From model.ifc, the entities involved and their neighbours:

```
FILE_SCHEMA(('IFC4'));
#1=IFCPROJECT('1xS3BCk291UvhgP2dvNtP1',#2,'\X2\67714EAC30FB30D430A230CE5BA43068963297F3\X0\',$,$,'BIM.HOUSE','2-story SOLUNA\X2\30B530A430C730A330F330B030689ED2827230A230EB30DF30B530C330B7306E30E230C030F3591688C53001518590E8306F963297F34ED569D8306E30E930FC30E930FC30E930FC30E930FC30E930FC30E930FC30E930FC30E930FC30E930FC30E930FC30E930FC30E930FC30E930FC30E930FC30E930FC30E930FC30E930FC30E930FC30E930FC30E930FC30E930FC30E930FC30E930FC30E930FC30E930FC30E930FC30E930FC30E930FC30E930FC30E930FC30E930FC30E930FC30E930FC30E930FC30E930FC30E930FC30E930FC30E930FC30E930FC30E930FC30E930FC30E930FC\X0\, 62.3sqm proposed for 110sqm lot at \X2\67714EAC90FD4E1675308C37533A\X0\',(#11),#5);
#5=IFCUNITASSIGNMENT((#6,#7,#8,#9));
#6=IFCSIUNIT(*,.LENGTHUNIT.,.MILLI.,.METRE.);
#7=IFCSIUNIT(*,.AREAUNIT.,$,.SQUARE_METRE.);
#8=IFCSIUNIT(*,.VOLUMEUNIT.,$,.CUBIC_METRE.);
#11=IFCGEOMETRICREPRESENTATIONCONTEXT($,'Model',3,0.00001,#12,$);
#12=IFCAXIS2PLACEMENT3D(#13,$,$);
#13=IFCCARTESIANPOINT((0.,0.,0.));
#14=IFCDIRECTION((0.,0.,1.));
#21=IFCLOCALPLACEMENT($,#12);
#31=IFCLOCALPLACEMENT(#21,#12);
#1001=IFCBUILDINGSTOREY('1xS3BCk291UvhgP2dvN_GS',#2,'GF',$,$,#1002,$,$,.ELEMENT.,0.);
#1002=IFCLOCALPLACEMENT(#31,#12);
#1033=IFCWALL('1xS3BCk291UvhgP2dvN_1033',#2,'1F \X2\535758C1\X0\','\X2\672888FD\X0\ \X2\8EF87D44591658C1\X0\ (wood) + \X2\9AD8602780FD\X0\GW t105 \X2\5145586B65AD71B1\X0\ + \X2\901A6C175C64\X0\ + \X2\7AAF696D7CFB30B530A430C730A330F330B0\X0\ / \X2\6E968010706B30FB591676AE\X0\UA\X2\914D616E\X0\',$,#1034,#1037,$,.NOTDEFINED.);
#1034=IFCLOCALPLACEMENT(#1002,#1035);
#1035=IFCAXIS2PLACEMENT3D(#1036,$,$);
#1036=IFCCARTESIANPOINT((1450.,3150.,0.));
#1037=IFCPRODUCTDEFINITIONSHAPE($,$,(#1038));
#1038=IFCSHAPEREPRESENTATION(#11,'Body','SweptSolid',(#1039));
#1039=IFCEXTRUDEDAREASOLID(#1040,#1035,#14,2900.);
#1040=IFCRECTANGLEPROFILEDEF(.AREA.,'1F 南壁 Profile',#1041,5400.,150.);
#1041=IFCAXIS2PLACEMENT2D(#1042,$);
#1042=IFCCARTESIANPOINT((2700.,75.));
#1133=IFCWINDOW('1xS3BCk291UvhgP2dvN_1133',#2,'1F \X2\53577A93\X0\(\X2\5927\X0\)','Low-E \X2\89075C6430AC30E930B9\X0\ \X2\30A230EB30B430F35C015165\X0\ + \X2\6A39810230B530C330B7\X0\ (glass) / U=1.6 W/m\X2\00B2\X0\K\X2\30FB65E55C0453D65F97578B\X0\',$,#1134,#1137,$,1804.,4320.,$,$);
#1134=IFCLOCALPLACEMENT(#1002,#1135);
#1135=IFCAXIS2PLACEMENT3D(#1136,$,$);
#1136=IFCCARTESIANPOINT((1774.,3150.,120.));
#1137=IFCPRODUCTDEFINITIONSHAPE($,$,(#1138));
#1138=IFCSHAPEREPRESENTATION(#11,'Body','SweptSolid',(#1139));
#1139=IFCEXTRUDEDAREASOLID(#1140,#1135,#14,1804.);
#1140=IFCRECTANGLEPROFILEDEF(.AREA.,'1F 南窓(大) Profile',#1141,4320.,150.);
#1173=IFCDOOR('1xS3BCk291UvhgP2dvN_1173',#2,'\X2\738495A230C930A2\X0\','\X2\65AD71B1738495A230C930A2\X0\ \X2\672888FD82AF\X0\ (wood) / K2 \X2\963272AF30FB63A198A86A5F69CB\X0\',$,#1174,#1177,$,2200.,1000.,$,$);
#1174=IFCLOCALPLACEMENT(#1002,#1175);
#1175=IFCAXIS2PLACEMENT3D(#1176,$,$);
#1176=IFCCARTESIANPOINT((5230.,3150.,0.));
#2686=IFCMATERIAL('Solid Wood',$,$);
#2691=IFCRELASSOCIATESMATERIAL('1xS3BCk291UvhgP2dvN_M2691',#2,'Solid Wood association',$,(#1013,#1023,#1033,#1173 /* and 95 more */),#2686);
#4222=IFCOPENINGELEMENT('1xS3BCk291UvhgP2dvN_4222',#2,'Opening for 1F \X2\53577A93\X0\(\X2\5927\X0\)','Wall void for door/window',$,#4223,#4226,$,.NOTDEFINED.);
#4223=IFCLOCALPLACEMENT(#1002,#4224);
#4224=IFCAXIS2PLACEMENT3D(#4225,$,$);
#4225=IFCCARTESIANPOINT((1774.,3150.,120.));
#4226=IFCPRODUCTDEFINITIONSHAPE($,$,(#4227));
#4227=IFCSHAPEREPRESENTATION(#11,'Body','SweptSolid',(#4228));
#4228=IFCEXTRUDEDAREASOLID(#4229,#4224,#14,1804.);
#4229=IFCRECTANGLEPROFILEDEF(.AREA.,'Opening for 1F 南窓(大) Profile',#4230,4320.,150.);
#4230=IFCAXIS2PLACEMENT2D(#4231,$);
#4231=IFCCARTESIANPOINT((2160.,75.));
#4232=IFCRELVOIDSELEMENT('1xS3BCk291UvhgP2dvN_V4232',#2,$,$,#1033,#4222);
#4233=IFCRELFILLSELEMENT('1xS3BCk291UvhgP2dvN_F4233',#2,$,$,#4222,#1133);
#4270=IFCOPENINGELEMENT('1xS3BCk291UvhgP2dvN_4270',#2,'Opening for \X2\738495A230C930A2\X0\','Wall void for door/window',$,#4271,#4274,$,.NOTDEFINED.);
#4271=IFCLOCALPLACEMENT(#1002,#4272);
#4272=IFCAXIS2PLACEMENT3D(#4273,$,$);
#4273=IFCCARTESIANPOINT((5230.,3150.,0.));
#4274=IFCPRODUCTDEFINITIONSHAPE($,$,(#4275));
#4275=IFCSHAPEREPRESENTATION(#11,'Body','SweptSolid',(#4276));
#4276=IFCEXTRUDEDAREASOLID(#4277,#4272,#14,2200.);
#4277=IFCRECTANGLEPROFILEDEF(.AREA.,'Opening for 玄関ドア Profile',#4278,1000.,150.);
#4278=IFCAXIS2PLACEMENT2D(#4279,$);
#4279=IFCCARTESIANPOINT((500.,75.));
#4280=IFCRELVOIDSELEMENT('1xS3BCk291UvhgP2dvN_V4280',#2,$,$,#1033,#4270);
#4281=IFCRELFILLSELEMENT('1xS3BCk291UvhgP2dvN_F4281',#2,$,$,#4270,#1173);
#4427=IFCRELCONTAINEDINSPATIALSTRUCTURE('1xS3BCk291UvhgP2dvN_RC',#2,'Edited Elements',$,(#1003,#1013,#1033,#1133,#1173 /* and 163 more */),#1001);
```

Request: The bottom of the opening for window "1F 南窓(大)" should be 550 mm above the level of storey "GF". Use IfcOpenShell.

```python
import numpy as np
import ifcopenshell
import ifcopenshell.api.geometry
import ifcopenshell.geom
import ifcopenshell.util.element
import ifcopenshell.util.placement
import ifcopenshell.util.shape
import ifcopenshell.util.unit

model = ifcopenshell.open("model.ifc")
unit_scale = ifcopenshell.util.unit.calculate_unit_scale(model)

window = model.by_guid("1xS3BCk291UvhgP2dvN_1133")
opening = window.FillsVoids[0].RelatingOpeningElement
storey = ifcopenshell.util.element.get_container(window, ifc_class="IfcBuildingStorey")
level = ifcopenshell.util.placement.get_local_placement(storey.ObjectPlacement)[2, 3]

# The opening's origin need not be at the sill, so measure its lowest point.
shape = ifcopenshell.geom.create_shape(ifcopenshell.geom.settings(), opening)
bottom = ifcopenshell.util.shape.get_shape_bottom_elevation(shape, shape.geometry) / unit_scale
dz = level + 0.55 / unit_scale - bottom

shift = np.array([0.0, 0.0, dz])
# The window is not placed relative to its opening, so move both.
for product in (opening, window):
    matrix = ifcopenshell.util.placement.get_local_placement(product.ObjectPlacement)
    matrix[:3, 3] += shift
    ifcopenshell.api.geometry.edit_object_placement(model, product=product, matrix=matrix, is_si=False)

print(f"moved by {dz * unit_scale:+.3f} m")

model.write("model-out.ifc")
```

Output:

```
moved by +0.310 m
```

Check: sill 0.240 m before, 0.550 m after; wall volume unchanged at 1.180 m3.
